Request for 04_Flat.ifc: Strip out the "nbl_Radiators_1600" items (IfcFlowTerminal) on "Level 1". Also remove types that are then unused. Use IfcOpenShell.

First a look at what the model holds.

```python
import ifcopenshell
import ifcopenshell.util.element

model = ifcopenshell.open("04_Flat.ifc")
print(model.schema)
storey = next(s for s in model.by_type("IfcBuildingStorey") if s.Name == "Level 1")
terminals = [e for e in ifcopenshell.util.element.get_decomposition(storey) if e.is_a("IfcFlowTerminal")]
seen = {}
for e in terminals:
    element_type = ifcopenshell.util.element.get_type(e)
    name = element_type.Name if element_type not in (None, e) else None
    seen[name] = seen.get(name, 0) + 1
for name, count in sorted(seen.items(), key=str):
    print(count, "x", name)
```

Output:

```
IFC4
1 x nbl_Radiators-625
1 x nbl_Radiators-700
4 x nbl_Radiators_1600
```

```python
import ifcopenshell
import ifcopenshell.api.root
import ifcopenshell.util.element

model = ifcopenshell.open("04_Flat.ifc")

storey = next(s for s in model.by_type("IfcBuildingStorey") if s.Name == "Level 1")
terminals = [e for e in ifcopenshell.util.element.get_decomposition(storey) if e.is_a("IfcFlowTerminal")]
targets = [e for e in terminals if (t := ifcopenshell.util.element.get_type(e)) not in (None, e) and t.Name == "nbl_Radiators_1600"]
types = {ifcopenshell.util.element.get_type(e) for e in targets} - {None, *targets}

for e in targets:
    ifcopenshell.api.root.remove_product(model, product=e)
print(len(targets), "removed")

unused = [t for t in types if not ifcopenshell.util.element.get_types(t)]
for t in unused:
    ifcopenshell.api.root.remove_product(model, product=t)
print(len(unused), "unused types removed")

model.write("04_Flat_updated.ifc")
```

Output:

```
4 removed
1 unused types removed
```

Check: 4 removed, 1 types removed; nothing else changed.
